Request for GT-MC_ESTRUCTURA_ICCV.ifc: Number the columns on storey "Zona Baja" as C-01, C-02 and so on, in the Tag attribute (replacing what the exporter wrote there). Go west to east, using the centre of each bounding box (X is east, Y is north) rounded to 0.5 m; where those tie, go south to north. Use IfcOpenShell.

First a look at what the model holds.

```python
import ifcopenshell
import ifcopenshell.util.element
import ifcopenshell.util.placement

model = ifcopenshell.open("GT-MC_ESTRUCTURA_ICCV.ifc")
print(model.schema)
storey = next(s for s in model.by_type("IfcBuildingStorey") if s.Name == "Zona Baja")
columns = [e for e in ifcopenshell.util.element.get_decomposition(storey) if e.is_a("IfcColumn")]
for e in sorted(columns, key=lambda e: e.id()):
    origin = ifcopenshell.util.placement.get_local_placement(e.ObjectPlacement)[:3, 3]
    print(e.id(), e.Tag, e.Name, origin.round(2) + 0.0, sep=" | ")
```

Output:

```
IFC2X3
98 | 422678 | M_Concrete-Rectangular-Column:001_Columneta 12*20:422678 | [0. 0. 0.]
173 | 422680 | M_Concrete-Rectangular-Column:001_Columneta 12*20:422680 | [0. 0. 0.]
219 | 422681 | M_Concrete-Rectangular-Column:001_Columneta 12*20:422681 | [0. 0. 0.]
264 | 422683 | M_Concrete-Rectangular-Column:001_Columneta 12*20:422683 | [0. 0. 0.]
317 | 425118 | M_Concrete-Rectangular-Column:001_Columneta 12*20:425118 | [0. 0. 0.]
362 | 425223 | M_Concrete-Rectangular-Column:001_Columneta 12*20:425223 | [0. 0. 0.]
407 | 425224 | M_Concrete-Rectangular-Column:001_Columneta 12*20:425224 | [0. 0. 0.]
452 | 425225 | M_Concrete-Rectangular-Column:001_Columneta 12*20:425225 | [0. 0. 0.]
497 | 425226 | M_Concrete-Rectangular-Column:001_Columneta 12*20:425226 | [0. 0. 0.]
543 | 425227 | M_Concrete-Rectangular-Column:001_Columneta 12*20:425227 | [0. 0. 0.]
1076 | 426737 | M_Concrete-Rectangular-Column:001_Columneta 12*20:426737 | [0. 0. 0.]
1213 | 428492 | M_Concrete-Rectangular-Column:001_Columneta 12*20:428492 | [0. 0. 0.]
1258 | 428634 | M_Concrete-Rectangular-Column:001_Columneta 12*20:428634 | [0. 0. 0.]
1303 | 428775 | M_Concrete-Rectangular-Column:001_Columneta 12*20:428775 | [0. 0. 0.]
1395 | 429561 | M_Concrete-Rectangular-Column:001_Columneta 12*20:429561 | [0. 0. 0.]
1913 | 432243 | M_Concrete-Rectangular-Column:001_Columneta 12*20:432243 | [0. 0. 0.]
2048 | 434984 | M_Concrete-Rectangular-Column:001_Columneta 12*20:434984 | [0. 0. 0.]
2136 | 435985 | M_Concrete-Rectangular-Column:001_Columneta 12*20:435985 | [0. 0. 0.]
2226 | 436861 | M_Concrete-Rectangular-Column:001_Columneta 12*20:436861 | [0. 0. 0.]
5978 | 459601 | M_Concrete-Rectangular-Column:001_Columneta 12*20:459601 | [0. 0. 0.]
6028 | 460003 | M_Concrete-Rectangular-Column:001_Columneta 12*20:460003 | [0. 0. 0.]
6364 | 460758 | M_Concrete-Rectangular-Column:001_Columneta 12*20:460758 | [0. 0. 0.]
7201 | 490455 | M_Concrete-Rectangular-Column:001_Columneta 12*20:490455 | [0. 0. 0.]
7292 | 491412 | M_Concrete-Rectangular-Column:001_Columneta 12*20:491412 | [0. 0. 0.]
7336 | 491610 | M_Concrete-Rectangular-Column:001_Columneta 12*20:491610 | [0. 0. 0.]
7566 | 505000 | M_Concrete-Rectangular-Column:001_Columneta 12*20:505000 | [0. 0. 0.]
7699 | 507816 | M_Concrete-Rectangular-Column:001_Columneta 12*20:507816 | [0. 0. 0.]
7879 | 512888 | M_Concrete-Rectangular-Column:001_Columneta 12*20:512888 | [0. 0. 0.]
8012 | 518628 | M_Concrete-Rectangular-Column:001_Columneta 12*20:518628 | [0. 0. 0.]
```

```python
import ifcopenshell
import ifcopenshell.geom
import ifcopenshell.util.element
import ifcopenshell.util.shape

model = ifcopenshell.open("GT-MC_ESTRUCTURA_ICCV.ifc")
settings = ifcopenshell.geom.settings()
settings.set("use-world-coords", True)


def centre(element):
    shape = ifcopenshell.geom.create_shape(settings, element)
    return ifcopenshell.util.shape.get_bbox_centroid(shape.geometry)


storey = next(s for s in model.by_type("IfcBuildingStorey") if s.Name == "Zona Baja")
columns = [e for e in ifcopenshell.util.element.get_decomposition(storey) if e.is_a("IfcColumn")]

# Insertion points can sit at a corner or the storey origin, so sort by the geometry (in metres).
centres = {e: centre(e) for e in columns}
columns.sort(key=lambda e: (round(centres[e][0] / 0.5), centres[e][1]))

for i, e in enumerate(columns, start=1):
    number = f"C-{i:02d}"
    e.Tag = number
    print(e.id(), number)

model.write("GT-MC_ESTRUCTURA_ICCV_v2.ifc")
```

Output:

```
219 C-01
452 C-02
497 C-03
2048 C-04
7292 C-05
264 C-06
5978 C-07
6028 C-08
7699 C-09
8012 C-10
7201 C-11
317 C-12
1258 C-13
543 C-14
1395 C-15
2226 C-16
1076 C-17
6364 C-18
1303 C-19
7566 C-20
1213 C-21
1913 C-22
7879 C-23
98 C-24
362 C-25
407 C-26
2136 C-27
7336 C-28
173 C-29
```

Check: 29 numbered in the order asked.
